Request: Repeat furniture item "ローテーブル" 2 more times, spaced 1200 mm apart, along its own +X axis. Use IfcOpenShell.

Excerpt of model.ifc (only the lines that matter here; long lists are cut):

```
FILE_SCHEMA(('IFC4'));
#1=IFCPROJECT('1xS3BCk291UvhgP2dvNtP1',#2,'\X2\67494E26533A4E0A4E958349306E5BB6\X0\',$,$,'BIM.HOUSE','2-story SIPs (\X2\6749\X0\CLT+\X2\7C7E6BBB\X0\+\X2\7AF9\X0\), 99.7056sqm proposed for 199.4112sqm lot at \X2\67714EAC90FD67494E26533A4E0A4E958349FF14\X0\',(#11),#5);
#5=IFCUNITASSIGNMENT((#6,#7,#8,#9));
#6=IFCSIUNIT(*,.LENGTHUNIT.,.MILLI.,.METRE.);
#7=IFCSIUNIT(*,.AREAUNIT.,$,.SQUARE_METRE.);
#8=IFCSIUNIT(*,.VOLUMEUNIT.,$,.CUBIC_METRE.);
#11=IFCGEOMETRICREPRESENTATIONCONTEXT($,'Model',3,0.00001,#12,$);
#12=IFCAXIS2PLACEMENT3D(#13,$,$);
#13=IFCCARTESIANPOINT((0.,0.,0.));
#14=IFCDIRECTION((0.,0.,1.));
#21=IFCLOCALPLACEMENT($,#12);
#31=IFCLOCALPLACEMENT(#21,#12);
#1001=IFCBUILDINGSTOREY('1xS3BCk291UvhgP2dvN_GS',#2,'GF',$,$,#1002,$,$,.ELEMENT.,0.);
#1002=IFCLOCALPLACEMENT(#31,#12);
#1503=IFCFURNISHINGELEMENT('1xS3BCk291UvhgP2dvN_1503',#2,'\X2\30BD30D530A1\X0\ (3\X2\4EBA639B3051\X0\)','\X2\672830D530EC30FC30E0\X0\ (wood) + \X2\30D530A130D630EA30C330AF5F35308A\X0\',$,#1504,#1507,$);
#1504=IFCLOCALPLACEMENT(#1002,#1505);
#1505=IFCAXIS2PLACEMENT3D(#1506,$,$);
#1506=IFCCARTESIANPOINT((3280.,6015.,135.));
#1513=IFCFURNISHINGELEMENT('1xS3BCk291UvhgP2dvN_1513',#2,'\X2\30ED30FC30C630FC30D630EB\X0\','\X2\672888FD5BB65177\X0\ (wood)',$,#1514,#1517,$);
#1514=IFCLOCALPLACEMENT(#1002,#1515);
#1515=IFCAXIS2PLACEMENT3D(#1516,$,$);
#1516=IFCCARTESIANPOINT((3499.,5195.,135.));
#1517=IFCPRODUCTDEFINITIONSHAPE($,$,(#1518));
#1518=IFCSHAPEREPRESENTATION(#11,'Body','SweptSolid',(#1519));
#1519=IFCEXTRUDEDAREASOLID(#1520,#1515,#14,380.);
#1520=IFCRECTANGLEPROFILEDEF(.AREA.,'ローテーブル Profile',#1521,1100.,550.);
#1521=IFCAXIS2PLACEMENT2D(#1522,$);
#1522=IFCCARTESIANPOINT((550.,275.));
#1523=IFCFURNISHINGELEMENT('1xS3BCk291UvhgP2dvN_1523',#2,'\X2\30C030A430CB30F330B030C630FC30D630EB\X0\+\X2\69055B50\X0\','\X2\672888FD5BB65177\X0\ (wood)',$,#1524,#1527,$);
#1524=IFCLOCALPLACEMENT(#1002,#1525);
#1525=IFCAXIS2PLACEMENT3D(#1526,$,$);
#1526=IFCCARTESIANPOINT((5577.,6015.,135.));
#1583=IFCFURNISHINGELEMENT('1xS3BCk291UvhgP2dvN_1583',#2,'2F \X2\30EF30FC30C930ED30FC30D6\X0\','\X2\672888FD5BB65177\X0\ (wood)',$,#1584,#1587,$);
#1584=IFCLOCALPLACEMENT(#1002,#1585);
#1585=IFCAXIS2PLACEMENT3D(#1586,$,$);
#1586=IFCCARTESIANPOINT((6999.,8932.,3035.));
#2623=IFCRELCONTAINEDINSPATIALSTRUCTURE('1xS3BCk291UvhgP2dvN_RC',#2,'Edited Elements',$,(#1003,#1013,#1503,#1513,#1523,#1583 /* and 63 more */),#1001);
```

```python
import ifcopenshell
import ifcopenshell.api.geometry
import ifcopenshell.api.root
import ifcopenshell.util.element
import ifcopenshell.util.placement
import ifcopenshell.util.unit

model = ifcopenshell.open("model.ifc")
unit_scale = ifcopenshell.util.unit.calculate_unit_scale(model)


def reuse_history(source, copy):
    """copy_class also copies each property set's owner history, people and application; keep the originals."""
    for rel in copy.IsDefinedBy:
        if rel.is_a("IfcRelDefinesByProperties") and (history := rel.RelatingPropertyDefinition.OwnerHistory):
            rel.RelatingPropertyDefinition.OwnerHistory = source.OwnerHistory
            ifcopenshell.util.element.remove_deep2(model, history)


source = model.by_guid("1xS3BCk291UvhgP2dvN_1513")
base = ifcopenshell.util.placement.get_local_placement(source.ObjectPlacement)
step = base[:3, 0] * 1.2 / unit_scale

for i in range(1, 3):
    copy = ifcopenshell.api.root.copy_class(model, product=source)
    copy.Representation = ifcopenshell.util.element.copy_deep(
        model, source.Representation, exclude=["IfcGeometricRepresentationContext", "IfcRepresentationMap"]
    )
    reuse_history(source, copy)
    matrix = base.copy()
    matrix[:3, 3] += i * step
    print("added at", matrix[:3, 3].round(3) + 0.0)
    ifcopenshell.api.geometry.edit_object_placement(model, product=copy, matrix=matrix, is_si=False)

model.write("model-out.ifc")
```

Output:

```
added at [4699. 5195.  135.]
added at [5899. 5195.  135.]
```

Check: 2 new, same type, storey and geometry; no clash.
